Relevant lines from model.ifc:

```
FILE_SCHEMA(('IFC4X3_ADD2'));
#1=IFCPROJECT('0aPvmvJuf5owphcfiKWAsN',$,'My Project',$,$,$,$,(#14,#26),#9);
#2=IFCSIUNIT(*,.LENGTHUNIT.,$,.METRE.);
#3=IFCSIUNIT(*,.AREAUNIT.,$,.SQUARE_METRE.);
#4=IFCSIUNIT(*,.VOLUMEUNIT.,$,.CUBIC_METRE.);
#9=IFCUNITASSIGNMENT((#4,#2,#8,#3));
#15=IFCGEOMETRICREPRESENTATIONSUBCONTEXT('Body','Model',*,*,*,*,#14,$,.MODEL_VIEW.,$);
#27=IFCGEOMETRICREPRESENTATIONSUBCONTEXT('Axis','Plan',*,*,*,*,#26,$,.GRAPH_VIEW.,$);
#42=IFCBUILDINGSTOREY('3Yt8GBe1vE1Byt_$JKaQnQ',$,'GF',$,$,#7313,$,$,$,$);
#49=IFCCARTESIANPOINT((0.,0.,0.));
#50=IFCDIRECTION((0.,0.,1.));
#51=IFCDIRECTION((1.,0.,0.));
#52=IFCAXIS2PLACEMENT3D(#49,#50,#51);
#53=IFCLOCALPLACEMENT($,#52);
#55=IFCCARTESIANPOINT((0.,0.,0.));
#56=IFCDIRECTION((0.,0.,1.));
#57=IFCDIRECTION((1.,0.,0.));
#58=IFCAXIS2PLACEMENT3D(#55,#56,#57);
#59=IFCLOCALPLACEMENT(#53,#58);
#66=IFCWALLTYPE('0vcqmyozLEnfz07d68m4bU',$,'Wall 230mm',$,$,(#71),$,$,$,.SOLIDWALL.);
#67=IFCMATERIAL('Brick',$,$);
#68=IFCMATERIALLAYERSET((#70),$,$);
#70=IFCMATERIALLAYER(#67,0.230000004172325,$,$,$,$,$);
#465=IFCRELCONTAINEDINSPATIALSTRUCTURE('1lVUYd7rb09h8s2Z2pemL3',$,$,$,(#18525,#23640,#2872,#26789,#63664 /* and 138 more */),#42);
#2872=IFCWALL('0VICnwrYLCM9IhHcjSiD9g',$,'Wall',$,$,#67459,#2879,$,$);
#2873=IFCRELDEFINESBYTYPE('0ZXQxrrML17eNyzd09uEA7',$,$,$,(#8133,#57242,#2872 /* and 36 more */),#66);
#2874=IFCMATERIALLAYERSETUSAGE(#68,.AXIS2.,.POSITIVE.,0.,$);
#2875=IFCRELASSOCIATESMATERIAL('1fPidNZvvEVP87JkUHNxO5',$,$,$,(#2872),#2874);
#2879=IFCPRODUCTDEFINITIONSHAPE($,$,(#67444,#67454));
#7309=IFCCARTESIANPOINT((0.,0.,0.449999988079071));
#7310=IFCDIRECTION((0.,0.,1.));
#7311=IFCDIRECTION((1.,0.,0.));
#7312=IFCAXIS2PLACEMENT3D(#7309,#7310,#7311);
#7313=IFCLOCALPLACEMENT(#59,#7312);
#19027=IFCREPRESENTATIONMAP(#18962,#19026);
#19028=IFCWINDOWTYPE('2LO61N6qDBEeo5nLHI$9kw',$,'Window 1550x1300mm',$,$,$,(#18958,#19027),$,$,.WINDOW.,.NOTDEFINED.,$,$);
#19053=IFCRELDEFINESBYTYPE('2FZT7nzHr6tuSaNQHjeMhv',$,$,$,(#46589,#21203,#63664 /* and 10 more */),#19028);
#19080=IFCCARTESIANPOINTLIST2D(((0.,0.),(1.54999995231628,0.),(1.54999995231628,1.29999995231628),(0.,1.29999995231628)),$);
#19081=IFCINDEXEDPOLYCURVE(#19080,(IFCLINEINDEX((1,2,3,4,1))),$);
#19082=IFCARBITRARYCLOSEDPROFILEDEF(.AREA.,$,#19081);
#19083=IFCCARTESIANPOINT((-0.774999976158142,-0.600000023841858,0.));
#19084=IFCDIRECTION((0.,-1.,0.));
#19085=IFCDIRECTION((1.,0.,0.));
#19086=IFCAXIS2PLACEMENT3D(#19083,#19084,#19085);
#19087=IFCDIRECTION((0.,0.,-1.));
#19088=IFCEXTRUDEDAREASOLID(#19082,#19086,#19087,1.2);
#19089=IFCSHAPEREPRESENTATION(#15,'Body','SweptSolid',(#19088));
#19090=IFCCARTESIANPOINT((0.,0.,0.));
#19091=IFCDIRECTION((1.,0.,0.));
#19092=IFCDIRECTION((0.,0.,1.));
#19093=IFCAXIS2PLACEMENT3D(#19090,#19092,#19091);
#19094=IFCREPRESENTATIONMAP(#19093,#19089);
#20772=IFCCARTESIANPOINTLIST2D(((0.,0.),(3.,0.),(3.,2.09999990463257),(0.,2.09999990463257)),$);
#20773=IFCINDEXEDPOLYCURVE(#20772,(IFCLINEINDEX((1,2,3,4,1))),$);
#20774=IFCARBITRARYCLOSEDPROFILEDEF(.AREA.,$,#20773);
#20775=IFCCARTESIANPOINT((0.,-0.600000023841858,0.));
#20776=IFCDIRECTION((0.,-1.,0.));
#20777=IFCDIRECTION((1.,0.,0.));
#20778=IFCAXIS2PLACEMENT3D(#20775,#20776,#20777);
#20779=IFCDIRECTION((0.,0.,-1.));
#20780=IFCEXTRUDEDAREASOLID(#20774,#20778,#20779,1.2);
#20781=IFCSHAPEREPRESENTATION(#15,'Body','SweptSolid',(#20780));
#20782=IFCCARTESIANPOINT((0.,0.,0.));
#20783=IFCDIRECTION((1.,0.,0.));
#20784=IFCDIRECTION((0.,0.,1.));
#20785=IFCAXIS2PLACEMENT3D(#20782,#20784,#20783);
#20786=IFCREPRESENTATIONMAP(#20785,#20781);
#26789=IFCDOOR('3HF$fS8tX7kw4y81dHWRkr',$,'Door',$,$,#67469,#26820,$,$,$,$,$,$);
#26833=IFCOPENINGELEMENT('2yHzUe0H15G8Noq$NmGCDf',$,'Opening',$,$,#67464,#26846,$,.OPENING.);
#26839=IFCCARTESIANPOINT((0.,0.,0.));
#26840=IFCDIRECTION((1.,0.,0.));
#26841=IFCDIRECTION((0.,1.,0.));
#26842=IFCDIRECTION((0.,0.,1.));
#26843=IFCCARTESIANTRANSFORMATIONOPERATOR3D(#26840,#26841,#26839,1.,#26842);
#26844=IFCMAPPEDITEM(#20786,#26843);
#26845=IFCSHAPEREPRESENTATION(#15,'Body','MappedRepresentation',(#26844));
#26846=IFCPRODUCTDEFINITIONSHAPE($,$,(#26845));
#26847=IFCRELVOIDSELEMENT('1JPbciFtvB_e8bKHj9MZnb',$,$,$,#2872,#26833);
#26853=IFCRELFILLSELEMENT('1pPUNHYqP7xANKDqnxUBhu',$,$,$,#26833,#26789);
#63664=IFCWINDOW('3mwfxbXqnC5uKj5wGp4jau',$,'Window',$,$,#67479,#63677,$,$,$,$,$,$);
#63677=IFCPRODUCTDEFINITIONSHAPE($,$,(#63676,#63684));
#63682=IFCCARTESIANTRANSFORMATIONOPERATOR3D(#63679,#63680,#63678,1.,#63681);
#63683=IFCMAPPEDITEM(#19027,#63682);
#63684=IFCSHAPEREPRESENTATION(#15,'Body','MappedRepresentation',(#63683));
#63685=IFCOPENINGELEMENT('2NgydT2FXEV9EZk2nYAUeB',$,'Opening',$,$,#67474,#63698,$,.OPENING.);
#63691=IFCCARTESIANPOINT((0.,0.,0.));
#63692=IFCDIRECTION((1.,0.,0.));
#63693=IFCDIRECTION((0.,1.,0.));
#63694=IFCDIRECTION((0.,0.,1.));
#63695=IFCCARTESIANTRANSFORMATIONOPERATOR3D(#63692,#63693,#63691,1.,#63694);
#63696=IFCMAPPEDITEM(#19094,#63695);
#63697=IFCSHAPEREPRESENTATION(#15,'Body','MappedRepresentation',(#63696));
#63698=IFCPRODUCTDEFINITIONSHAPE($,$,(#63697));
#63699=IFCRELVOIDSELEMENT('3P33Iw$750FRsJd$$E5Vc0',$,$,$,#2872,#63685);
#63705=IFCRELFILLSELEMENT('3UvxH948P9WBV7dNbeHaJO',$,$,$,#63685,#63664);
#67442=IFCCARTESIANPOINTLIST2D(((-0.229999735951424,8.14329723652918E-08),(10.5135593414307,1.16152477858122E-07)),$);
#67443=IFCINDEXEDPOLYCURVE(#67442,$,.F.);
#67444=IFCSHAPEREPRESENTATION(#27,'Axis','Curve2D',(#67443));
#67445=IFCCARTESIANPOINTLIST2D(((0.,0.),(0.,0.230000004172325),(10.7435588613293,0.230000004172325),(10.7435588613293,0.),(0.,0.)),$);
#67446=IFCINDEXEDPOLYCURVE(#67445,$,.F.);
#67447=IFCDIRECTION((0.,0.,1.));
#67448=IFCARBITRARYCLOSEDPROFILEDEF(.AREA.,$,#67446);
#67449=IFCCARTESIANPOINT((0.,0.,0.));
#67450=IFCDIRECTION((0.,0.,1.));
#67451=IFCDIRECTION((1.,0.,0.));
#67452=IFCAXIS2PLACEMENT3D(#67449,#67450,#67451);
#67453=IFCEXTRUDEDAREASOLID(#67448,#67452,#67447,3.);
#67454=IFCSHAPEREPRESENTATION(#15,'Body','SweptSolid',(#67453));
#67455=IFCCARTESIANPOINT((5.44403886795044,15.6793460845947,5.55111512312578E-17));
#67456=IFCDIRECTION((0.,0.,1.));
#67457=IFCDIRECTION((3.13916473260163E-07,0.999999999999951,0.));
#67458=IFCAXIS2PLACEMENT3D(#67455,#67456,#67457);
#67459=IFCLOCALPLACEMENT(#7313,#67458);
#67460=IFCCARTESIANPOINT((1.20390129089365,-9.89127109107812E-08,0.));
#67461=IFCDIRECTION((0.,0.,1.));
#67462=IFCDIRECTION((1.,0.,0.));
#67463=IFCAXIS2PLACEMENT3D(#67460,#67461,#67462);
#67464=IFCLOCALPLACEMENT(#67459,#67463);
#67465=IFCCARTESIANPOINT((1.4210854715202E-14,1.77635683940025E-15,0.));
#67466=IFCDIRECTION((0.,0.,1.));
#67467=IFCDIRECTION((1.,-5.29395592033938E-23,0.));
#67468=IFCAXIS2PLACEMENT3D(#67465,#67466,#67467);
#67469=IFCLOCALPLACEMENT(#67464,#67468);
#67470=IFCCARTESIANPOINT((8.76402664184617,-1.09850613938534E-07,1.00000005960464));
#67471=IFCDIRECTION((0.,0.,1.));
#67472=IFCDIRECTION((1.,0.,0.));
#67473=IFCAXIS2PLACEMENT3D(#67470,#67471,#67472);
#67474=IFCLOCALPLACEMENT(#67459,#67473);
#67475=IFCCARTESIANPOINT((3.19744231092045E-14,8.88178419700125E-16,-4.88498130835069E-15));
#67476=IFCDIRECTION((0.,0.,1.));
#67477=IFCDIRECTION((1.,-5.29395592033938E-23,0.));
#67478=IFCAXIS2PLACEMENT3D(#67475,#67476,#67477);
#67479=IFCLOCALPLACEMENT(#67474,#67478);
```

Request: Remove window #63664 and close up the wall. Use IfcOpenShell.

```python
import ifcopenshell
import ifcopenshell.api.feature
import ifcopenshell.api.root
import ifcopenshell.geom
import ifcopenshell.util.shape

model = ifcopenshell.open("model.ifc")
settings = ifcopenshell.geom.settings()


def volume(element):
    """Net volume in cubic metres, openings subtracted."""
    shape = ifcopenshell.geom.create_shape(settings, element)
    return ifcopenshell.util.shape.get_volume(shape.geometry)


window = model.by_guid("3mwfxbXqnC5uKj5wGp4jau")
opening = window.FillsVoids[0].RelatingOpeningElement
wall = opening.VoidsElements[0].RelatingBuildingElement
before = volume(wall)

ifcopenshell.api.root.remove_product(model, product=window)
ifcopenshell.api.feature.remove_feature(model, feature=opening)

after = volume(wall)

print(f"wall volume {before:.3f} -> {after:.3f} m3")

model.write("model-out.ifc")
```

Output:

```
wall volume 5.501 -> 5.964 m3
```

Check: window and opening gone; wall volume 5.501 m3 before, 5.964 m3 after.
